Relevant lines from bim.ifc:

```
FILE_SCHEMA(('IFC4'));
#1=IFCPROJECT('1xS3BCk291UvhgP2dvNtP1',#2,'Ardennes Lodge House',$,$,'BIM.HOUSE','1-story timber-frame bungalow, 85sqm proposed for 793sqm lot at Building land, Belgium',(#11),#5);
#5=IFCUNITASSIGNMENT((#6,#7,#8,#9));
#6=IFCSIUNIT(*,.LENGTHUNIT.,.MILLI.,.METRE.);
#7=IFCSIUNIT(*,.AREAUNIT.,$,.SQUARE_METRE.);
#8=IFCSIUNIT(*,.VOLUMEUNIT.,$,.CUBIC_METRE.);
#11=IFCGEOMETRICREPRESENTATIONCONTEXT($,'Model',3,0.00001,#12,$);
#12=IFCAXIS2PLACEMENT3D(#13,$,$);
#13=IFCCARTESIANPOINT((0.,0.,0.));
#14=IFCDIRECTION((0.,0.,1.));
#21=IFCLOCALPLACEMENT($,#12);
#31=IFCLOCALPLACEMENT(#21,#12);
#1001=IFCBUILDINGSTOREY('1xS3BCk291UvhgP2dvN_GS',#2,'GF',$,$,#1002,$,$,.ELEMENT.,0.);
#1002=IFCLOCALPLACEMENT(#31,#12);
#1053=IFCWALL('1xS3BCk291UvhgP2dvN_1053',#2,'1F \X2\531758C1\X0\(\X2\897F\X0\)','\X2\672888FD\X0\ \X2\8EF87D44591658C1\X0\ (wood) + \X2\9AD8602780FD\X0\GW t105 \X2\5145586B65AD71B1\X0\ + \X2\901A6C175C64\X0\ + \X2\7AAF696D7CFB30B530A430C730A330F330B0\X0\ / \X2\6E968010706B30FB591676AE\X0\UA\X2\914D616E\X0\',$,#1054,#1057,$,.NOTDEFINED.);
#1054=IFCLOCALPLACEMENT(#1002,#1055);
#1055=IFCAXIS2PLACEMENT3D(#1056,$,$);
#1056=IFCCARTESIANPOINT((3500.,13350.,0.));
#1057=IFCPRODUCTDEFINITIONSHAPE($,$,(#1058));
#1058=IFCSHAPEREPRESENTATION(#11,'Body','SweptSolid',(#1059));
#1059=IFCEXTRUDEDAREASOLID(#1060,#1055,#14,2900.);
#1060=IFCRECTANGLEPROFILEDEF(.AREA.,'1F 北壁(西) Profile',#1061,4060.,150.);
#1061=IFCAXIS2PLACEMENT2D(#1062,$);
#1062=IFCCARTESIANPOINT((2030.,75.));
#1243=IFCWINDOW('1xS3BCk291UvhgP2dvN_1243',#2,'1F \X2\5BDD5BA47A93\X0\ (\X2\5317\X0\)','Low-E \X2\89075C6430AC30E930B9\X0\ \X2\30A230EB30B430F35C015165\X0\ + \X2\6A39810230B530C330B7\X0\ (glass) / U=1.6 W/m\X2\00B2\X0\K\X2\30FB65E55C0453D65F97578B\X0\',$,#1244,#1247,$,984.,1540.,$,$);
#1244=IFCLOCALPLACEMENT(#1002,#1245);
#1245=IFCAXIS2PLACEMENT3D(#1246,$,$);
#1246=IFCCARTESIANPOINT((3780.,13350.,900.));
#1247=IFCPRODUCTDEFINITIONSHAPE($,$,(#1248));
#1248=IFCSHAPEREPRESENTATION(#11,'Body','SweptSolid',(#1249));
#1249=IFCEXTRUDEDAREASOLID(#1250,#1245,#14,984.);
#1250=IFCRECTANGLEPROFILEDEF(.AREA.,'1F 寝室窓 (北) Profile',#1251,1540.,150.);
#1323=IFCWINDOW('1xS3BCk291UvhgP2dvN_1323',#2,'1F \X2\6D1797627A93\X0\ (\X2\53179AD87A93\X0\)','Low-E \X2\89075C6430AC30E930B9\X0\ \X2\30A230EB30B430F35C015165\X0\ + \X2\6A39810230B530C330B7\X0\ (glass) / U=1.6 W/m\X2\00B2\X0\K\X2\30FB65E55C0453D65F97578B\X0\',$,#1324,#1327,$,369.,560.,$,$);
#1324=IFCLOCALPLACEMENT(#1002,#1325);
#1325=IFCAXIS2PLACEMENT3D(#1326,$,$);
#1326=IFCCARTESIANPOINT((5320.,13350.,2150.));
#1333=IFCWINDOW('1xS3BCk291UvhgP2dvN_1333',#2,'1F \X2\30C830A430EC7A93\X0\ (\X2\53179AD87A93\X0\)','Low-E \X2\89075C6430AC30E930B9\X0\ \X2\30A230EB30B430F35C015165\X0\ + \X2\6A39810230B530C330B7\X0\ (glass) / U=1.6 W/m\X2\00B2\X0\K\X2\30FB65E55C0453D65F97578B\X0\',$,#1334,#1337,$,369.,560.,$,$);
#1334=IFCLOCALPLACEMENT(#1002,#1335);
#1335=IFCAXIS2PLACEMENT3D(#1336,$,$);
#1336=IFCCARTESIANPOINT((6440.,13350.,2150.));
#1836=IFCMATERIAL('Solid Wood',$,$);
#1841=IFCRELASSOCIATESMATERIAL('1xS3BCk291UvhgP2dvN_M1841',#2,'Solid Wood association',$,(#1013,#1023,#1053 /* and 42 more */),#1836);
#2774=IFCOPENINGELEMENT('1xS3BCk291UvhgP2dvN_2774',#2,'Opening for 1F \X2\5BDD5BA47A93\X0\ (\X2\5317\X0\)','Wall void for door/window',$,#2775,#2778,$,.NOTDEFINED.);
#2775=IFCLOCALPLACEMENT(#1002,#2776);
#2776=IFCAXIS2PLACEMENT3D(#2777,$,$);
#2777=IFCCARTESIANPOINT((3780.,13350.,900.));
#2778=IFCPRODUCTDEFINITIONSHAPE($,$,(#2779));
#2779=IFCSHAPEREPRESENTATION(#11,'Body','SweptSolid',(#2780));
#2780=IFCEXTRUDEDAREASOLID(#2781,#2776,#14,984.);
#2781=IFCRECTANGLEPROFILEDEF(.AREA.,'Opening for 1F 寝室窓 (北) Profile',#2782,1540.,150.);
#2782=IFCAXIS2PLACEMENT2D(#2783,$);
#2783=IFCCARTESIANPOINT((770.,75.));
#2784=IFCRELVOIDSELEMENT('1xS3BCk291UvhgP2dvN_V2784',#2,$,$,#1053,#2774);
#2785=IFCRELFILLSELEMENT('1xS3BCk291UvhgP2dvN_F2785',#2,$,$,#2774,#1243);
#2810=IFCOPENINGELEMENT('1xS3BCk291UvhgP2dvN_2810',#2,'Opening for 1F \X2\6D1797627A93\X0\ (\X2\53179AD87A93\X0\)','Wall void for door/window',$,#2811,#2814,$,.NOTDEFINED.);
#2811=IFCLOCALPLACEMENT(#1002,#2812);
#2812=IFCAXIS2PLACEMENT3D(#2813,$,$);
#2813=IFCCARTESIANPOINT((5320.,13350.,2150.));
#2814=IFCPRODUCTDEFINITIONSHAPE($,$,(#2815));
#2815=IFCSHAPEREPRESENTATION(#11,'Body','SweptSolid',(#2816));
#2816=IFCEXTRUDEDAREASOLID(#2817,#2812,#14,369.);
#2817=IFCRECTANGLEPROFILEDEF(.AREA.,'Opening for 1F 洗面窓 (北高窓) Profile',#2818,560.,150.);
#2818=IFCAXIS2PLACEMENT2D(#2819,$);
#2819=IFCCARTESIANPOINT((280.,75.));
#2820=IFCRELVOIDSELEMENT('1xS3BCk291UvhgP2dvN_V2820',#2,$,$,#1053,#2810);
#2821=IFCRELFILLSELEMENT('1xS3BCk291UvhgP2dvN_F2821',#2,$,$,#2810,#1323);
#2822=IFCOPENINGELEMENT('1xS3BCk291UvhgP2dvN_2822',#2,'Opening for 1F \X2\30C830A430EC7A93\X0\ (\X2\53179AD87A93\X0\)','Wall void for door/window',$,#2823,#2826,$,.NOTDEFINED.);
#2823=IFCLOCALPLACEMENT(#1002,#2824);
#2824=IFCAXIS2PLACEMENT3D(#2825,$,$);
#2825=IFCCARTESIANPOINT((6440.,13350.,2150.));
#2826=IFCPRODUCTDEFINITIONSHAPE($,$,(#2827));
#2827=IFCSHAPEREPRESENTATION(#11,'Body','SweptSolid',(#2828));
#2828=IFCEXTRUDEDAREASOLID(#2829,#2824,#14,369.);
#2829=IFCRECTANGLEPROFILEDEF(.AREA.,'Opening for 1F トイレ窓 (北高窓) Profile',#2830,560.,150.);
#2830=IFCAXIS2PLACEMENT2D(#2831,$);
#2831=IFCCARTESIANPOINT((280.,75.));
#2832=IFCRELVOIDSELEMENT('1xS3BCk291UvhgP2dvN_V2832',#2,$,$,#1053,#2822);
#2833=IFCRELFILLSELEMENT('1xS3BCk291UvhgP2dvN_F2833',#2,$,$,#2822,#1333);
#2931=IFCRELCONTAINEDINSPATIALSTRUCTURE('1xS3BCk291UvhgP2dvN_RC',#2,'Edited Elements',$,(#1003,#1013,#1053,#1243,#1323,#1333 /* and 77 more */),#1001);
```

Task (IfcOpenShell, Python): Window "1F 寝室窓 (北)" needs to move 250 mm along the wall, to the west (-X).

```python
import ifcopenshell
import ifcopenshell.api.geometry
import ifcopenshell.util.placement
import ifcopenshell.util.unit

model = ifcopenshell.open("bim.ifc")
unit_scale = ifcopenshell.util.unit.calculate_unit_scale(model)

window = model.by_guid("1xS3BCk291UvhgP2dvN_1243")
opening = window.FillsVoids[0].RelatingOpeningElement
wall = opening.VoidsElements[0].RelatingBuildingElement

wall_matrix = ifcopenshell.util.placement.get_local_placement(wall.ObjectPlacement)
shift = wall_matrix[:3, 0] * -0.25 / unit_scale
before = ifcopenshell.util.placement.get_local_placement(window.ObjectPlacement)[:3, 3].copy()

# The window is not placed relative to its opening, so move both.
for product in (opening, window):
    matrix = ifcopenshell.util.placement.get_local_placement(product.ObjectPlacement)
    matrix[:3, 3] += shift
    ifcopenshell.api.geometry.edit_object_placement(model, product=product, matrix=matrix, is_si=False)

after = ifcopenshell.util.placement.get_local_placement(window.ObjectPlacement)[:3, 3]
print("window moved by", (after - before).round(3) + 0.0)

model.write("bim-out.ifc")
```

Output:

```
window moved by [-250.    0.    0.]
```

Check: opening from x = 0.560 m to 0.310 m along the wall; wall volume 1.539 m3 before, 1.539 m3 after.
